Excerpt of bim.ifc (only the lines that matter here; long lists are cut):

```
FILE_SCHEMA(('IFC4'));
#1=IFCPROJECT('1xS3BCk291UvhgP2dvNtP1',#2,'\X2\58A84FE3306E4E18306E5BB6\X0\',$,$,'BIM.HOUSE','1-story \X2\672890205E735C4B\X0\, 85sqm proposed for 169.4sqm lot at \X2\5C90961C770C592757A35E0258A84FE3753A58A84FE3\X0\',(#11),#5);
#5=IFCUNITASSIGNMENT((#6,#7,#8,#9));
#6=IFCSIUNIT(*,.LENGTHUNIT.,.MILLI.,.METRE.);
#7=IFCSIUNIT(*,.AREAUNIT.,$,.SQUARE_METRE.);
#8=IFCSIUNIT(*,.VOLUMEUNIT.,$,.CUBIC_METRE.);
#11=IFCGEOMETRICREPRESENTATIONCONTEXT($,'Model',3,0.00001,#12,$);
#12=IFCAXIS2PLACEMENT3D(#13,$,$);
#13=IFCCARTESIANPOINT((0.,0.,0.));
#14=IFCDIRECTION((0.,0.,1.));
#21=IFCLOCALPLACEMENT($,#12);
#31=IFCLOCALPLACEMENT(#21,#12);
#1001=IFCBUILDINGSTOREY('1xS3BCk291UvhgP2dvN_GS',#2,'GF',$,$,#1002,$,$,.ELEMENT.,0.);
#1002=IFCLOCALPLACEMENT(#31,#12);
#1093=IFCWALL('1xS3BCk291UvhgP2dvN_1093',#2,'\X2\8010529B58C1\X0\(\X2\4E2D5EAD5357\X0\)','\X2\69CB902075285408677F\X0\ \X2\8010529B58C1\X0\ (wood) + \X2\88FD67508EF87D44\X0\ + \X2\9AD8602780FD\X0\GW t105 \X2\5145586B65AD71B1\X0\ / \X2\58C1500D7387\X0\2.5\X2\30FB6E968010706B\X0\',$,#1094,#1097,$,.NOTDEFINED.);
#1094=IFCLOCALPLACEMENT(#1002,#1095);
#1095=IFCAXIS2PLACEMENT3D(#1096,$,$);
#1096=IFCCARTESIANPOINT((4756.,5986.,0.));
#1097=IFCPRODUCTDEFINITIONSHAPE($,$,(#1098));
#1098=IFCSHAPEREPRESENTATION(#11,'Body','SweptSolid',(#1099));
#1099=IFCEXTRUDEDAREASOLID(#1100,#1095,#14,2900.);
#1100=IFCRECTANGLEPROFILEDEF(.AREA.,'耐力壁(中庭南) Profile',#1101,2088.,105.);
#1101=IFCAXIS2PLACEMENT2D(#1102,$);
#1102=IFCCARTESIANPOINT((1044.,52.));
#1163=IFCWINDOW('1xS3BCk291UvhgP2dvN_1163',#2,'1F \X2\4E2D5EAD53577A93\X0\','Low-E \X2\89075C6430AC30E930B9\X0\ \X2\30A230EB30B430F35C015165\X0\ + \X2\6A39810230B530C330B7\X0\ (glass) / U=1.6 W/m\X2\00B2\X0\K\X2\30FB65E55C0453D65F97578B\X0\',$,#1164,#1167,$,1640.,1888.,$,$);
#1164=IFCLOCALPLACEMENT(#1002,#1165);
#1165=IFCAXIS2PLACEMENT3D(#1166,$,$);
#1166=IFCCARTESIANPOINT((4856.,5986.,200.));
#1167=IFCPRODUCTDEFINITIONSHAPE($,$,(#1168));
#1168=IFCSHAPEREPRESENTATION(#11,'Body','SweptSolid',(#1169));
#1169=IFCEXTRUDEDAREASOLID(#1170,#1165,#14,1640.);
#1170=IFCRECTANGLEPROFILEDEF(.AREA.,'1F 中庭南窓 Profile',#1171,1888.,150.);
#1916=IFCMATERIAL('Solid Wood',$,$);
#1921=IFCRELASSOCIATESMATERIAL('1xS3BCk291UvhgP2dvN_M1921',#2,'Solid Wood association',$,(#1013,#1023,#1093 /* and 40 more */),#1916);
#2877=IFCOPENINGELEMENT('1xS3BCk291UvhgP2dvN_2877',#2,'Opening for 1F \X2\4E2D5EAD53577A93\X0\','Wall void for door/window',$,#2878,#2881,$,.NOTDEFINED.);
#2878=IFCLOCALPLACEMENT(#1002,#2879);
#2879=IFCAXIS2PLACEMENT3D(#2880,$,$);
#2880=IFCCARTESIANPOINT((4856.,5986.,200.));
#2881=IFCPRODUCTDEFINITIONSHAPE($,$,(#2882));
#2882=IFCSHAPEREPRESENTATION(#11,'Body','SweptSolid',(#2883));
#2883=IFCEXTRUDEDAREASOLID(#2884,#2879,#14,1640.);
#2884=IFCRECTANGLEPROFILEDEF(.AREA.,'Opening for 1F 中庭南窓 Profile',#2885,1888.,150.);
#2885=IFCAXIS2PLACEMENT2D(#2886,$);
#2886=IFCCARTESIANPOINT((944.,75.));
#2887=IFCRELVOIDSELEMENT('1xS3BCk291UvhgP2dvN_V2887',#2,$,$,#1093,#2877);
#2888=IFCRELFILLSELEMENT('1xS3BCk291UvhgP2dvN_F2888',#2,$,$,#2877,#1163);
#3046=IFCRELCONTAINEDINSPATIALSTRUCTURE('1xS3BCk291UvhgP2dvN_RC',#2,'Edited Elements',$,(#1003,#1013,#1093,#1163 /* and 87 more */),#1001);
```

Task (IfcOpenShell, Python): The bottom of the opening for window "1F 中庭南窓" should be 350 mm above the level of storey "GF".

```python
import numpy as np
import ifcopenshell
import ifcopenshell.api.geometry
import ifcopenshell.geom
import ifcopenshell.util.element
import ifcopenshell.util.placement
import ifcopenshell.util.shape
import ifcopenshell.util.unit

model = ifcopenshell.open("bim.ifc")
unit_scale = ifcopenshell.util.unit.calculate_unit_scale(model)

window = model.by_guid("1xS3BCk291UvhgP2dvN_1163")
opening = window.FillsVoids[0].RelatingOpeningElement
storey = ifcopenshell.util.element.get_container(window, ifc_class="IfcBuildingStorey")
level = ifcopenshell.util.placement.get_local_placement(storey.ObjectPlacement)[2, 3]

# The opening's origin need not be at the sill, so measure its lowest point.
shape = ifcopenshell.geom.create_shape(ifcopenshell.geom.settings(), opening)
bottom = ifcopenshell.util.shape.get_shape_bottom_elevation(shape, shape.geometry) / unit_scale
dz = level + 0.35 / unit_scale - bottom

shift = np.array([0.0, 0.0, dz])
# The window is not placed relative to its opening, so move both.
for product in (opening, window):
    matrix = ifcopenshell.util.placement.get_local_placement(product.ObjectPlacement)
    matrix[:3, 3] += shift
    ifcopenshell.api.geometry.edit_object_placement(model, product=product, matrix=matrix, is_si=False)

print(f"moved by {dz * unit_scale:+.3f} m")

model.write("bim_updated.ifc")
```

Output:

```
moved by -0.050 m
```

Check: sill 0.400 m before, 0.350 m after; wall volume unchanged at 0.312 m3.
